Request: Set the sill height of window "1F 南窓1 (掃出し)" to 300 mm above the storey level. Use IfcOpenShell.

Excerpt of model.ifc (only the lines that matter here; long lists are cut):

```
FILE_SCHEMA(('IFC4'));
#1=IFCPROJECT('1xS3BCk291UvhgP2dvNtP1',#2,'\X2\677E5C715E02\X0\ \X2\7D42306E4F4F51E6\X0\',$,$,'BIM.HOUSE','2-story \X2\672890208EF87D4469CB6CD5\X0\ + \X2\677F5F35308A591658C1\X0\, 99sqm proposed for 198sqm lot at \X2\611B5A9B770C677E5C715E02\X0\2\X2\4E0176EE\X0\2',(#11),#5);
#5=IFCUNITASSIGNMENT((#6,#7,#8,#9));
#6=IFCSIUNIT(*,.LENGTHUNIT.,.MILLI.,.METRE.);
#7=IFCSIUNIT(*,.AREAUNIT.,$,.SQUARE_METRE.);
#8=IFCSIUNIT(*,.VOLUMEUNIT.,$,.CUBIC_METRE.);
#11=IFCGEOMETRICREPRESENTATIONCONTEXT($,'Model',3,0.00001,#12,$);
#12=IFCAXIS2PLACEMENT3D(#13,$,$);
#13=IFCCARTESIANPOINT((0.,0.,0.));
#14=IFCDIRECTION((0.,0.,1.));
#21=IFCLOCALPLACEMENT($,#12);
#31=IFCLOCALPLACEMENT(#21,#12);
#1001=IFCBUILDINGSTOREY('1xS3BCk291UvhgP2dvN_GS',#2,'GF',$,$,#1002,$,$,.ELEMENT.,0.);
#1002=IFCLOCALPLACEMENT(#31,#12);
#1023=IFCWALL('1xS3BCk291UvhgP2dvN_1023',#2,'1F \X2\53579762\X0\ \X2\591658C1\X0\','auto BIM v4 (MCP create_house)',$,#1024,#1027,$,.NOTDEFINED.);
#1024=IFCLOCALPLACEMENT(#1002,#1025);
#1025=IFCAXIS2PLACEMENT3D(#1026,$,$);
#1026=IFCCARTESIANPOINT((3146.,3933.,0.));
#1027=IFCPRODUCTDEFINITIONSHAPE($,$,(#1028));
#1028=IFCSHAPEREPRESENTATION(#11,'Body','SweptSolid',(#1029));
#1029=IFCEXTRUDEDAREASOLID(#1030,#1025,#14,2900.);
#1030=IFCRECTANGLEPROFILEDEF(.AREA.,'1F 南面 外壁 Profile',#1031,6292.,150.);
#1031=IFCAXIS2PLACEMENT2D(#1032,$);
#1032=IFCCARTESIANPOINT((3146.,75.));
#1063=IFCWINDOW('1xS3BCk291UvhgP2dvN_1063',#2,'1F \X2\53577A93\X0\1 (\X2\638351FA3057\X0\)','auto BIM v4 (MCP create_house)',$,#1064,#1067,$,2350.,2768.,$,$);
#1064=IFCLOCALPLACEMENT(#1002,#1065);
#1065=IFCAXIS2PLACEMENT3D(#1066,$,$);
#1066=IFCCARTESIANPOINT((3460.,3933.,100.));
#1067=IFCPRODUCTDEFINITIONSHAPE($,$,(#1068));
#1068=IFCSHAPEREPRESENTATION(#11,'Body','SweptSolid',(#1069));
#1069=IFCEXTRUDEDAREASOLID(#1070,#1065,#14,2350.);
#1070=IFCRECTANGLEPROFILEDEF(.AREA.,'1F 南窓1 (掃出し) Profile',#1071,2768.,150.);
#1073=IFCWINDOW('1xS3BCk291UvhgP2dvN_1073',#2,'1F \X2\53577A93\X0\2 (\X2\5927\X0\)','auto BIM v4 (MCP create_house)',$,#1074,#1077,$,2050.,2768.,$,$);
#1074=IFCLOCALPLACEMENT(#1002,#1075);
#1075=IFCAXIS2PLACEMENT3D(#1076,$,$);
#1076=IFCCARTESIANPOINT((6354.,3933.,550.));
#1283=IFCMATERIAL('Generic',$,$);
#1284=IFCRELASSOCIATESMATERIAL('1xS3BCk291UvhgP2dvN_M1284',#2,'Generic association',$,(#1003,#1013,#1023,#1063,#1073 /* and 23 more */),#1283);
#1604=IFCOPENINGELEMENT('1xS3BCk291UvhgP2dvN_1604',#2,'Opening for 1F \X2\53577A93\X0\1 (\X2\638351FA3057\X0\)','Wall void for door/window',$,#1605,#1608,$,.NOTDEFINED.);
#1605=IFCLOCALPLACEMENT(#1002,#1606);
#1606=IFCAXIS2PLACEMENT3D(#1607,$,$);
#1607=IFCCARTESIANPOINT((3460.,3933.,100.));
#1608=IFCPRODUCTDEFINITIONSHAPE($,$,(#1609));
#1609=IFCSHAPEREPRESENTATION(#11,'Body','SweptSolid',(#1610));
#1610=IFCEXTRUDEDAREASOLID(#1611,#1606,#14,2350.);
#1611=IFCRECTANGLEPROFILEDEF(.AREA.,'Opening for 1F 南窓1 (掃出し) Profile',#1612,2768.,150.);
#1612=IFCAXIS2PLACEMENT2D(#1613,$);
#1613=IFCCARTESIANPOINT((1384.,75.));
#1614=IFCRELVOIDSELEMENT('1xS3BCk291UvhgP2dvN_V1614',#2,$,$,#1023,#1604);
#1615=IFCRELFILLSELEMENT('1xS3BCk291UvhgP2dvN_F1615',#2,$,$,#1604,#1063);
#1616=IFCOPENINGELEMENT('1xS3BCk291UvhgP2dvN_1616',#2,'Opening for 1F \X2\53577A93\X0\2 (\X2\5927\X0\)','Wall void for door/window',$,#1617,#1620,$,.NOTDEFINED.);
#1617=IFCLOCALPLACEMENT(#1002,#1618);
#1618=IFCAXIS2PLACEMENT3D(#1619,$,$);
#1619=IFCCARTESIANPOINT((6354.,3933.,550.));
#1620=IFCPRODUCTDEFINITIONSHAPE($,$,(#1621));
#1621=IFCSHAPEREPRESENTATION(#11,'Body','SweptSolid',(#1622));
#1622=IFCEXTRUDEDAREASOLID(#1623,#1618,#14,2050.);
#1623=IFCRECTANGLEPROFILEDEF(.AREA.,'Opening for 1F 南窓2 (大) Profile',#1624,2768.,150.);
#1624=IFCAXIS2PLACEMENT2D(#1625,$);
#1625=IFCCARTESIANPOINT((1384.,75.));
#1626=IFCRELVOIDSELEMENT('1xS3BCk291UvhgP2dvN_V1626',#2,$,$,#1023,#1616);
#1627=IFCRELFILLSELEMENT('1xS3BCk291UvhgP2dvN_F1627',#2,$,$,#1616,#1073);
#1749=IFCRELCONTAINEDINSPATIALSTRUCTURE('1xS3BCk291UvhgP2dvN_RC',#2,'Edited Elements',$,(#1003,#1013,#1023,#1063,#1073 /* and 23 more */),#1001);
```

```python
import numpy as np
import ifcopenshell
import ifcopenshell.api.geometry
import ifcopenshell.geom
import ifcopenshell.util.element
import ifcopenshell.util.placement
import ifcopenshell.util.shape
import ifcopenshell.util.unit

model = ifcopenshell.open("model.ifc")
unit_scale = ifcopenshell.util.unit.calculate_unit_scale(model)

window = model.by_guid("1xS3BCk291UvhgP2dvN_1063")
opening = window.FillsVoids[0].RelatingOpeningElement
storey = ifcopenshell.util.element.get_container(window, ifc_class="IfcBuildingStorey")
level = ifcopenshell.util.placement.get_local_placement(storey.ObjectPlacement)[2, 3]

# The opening's origin need not be at the sill, so measure its lowest point.
shape = ifcopenshell.geom.create_shape(ifcopenshell.geom.settings(), opening)
bottom = ifcopenshell.util.shape.get_shape_bottom_elevation(shape, shape.geometry) / unit_scale
dz = level + 300.0 - bottom

shift = np.array([0.0, 0.0, dz])
# The window is not placed relative to its opening, so move both.
for product in (opening, window):
    matrix = ifcopenshell.util.placement.get_local_placement(product.ObjectPlacement)
    matrix[:3, 3] += shift
    ifcopenshell.api.geometry.edit_object_placement(model, product=product, matrix=matrix, is_si=False)

print(f"moved by {dz * unit_scale:+.3f} m")

model.write("model_rev.ifc")
```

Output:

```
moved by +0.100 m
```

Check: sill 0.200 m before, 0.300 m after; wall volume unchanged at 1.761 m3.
